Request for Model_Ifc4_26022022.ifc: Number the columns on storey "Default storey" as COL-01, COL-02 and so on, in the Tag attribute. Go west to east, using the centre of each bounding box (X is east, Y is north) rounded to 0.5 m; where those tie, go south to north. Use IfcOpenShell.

First a look at what the model holds.

```python
import ifcopenshell
import ifcopenshell.util.element
import ifcopenshell.util.placement

model = ifcopenshell.open("Model_Ifc4_26022022.ifc")
print(model.schema)
storey = next(s for s in model.by_type("IfcBuildingStorey") if s.Name == "Default storey")
columns = [e for e in ifcopenshell.util.element.get_decomposition(storey) if e.is_a("IfcColumn")]
for e in sorted(columns, key=lambda e: e.id()):
    origin = ifcopenshell.util.placement.get_local_placement(e.ObjectPlacement)[:3, 3]
    print(e.id(), e.Tag, e.Name, origin.round(2) + 0.0, sep=" | ")
```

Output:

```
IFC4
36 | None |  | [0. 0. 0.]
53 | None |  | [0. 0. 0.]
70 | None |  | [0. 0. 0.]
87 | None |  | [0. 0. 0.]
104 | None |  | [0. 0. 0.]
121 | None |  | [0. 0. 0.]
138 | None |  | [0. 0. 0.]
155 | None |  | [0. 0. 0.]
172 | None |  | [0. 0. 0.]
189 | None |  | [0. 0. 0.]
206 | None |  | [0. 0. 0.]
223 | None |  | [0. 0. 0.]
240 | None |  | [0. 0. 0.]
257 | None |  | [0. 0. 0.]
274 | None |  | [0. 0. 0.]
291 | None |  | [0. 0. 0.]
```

```python
import ifcopenshell
import ifcopenshell.geom
import ifcopenshell.util.element
import ifcopenshell.util.shape

model = ifcopenshell.open("Model_Ifc4_26022022.ifc")
settings = ifcopenshell.geom.settings()
settings.set("use-world-coords", True)


def centre(element):
    shape = ifcopenshell.geom.create_shape(settings, element)
    return ifcopenshell.util.shape.get_bbox_centroid(shape.geometry)


storey = next(s for s in model.by_type("IfcBuildingStorey") if s.Name == "Default storey")
columns = [e for e in ifcopenshell.util.element.get_decomposition(storey) if e.is_a("IfcColumn")]

# Insertion points can sit at a corner or the storey origin, so sort by the geometry (in metres).
centres = {e: centre(e) for e in columns}
columns.sort(key=lambda e: (round(centres[e][0] / 0.5), centres[e][1]))

for i, e in enumerate(columns, start=1):
    number = f"COL-{i:02d}"
    e.Tag = number
    print(e.id(), number)

model.write("Model_Ifc4_26022022_edited.ifc")
```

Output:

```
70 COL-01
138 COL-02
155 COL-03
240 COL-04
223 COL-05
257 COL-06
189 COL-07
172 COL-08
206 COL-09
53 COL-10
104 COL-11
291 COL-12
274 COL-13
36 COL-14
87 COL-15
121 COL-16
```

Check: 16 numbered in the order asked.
